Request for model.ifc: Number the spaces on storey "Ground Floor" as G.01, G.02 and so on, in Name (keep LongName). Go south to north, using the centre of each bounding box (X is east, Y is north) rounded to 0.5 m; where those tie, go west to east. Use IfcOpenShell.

First a look at what the model holds.

```python
import ifcopenshell
import ifcopenshell.util.element
import ifcopenshell.util.placement

model = ifcopenshell.open("model.ifc")
print(model.schema)
storey = next(s for s in model.by_type("IfcBuildingStorey") if s.Name == "Ground Floor")
spaces = [e for e in ifcopenshell.util.element.get_decomposition(storey) if e.is_a("IfcSpace")]
for e in sorted(spaces, key=lambda e: e.id()):
    origin = ifcopenshell.util.placement.get_local_placement(e.ObjectPlacement)[:3, 3]
    print(e.id(), e.Name, e.LongName, origin.round(2) + 0.0, sep=" | ")
```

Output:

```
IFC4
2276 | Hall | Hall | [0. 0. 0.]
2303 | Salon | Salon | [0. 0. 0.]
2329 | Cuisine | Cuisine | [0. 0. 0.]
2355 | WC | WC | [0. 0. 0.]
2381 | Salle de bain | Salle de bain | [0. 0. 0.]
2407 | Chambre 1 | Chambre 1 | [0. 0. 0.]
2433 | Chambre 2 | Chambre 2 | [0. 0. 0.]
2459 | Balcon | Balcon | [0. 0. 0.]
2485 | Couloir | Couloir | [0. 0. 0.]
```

```python
import ifcopenshell
import ifcopenshell.geom
import ifcopenshell.util.element
import ifcopenshell.util.shape

model = ifcopenshell.open("model.ifc")
settings = ifcopenshell.geom.settings()
settings.set("use-world-coords", True)


def centre(element):
    shape = ifcopenshell.geom.create_shape(settings, element)
    return ifcopenshell.util.shape.get_bbox_centroid(shape.geometry)


storey = next(s for s in model.by_type("IfcBuildingStorey") if s.Name == "Ground Floor")
spaces = [e for e in ifcopenshell.util.element.get_decomposition(storey) if e.is_a("IfcSpace")]

# Insertion points can sit at a corner or the storey origin, so sort by the geometry (in metres).
centres = {e: centre(e) for e in spaces}
spaces.sort(key=lambda e: (round(centres[e][1] / 0.5), centres[e][0]))

for i, e in enumerate(spaces, start=1):
    number = f"G.{i:02d}"
    e.Name = number
    print(e.id(), number)

model.write("model-out.ifc")
```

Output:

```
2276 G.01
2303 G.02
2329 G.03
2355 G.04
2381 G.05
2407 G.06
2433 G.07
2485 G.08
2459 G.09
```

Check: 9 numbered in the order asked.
